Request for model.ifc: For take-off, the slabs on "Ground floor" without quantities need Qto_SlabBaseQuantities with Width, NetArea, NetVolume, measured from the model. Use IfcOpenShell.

First a look at what the model holds.

```python
import ifcopenshell
import ifcopenshell.util.element
import ifcopenshell.util.unit

model = ifcopenshell.open("model.ifc")
print(model.schema)
for unit_type in ("LENGTHUNIT", "AREAUNIT", "VOLUMEUNIT"):
    print(unit_type, ifcopenshell.util.unit.calculate_unit_scale(model, unit_type))
storey = next(s for s in model.by_type("IfcBuildingStorey") if s.Name == "Ground floor")
slabs = [e for e in ifcopenshell.util.element.get_decomposition(storey) if e.is_a("IfcSlab")]
for e in sorted(slabs, key=lambda e: e.id()):
    print(e.id(), e.is_a(), e.Name, list(ifcopenshell.util.element.get_psets(e, qtos_only=True)), sep=" | ")
```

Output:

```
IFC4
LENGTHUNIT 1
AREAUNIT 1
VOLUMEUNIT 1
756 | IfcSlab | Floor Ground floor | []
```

```python
import ifcopenshell
import ifcopenshell.api.pset
import ifcopenshell.geom
import ifcopenshell.util.element
import ifcopenshell.util.shape
import ifcopenshell.util.unit

model = ifcopenshell.open("model.ifc")
unit_scale = ifcopenshell.util.unit.calculate_unit_scale(model)
area_scale = ifcopenshell.util.unit.calculate_unit_scale(model, "AREAUNIT")
volume_scale = ifcopenshell.util.unit.calculate_unit_scale(model, "VOLUMEUNIT")
settings = ifcopenshell.geom.settings()

storey = next(s for s in model.by_type("IfcBuildingStorey") if s.Name == "Ground floor")
slabs = [e for e in ifcopenshell.util.element.get_decomposition(storey) if e.is_a("IfcSlab")]

for e in sorted(slabs, key=lambda e: e.id()):
    if ifcopenshell.util.element.get_psets(e, qtos_only=True, should_inherit=False):
        continue
    # Geometry comes back in metres, in the element's own axes.
    shape = ifcopenshell.geom.create_shape(settings, e)
    values = {
        "Width": ifcopenshell.util.shape.get_z(shape.geometry) / unit_scale,
        "NetArea": ifcopenshell.util.shape.get_footprint_area(shape.geometry) / area_scale,
        "NetVolume": ifcopenshell.util.shape.get_volume(shape.geometry) / volume_scale,
    }
    qto = ifcopenshell.api.pset.add_qto(model, product=e, name="Qto_SlabBaseQuantities")
    ifcopenshell.api.pset.edit_qto(model, qto=qto, properties=values)
    print(e.id(), {k: round(v, 3) for k, v in values.items()})

model.write("model_v2.ifc")
```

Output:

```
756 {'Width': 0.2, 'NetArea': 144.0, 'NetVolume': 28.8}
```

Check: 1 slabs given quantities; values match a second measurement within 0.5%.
